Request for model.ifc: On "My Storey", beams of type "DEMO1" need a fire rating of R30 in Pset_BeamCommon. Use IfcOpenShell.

First a look at what the model holds.

```python
import ifcopenshell
import ifcopenshell.util.element

model = ifcopenshell.open("model.ifc")
print(model.schema)
storey = next(s for s in model.by_type("IfcBuildingStorey") if s.Name == "My Storey")
beams = [e for e in ifcopenshell.util.element.get_decomposition(storey) if e.is_a("IfcBeam")]
seen = {}
for e in beams:
    element_type = ifcopenshell.util.element.get_type(e)
    key = (element_type.Name if element_type != e and element_type else None, ifcopenshell.util.element.get_pset(e, "Pset_BeamCommon", "FireRating"))
    seen[key] = seen.get(key, 0) + 1
for (name, value), count in sorted(seen.items(), key=str):
    print(count, "x", name, "|", value)
```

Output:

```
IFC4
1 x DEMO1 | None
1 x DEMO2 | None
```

```python
import ifcopenshell
import ifcopenshell.api.pset
import ifcopenshell.util.element

model = ifcopenshell.open("model.ifc")

storey = next(s for s in model.by_type("IfcBuildingStorey") if s.Name == "My Storey")
beams = [e for e in ifcopenshell.util.element.get_decomposition(storey) if e.is_a("IfcBeam")]

count = 0
for e in beams:
    element_type = ifcopenshell.util.element.get_type(e)
    if element_type in (None, e) or element_type.Name != "DEMO1":
        continue
    # add_pset returns the element's existing set when there is one.
    pset = ifcopenshell.api.pset.add_pset(model, product=e, name="Pset_BeamCommon")
    ifcopenshell.api.pset.edit_pset(model, pset=pset, properties={"FireRating": "R30"})
    count += 1

print(count, "beams updated")

model.write("model_rev.ifc")
```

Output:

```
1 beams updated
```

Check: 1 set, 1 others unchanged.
